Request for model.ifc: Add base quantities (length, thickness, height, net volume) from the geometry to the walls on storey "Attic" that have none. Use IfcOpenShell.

First a look at what the model holds.

```python
import ifcopenshell
import ifcopenshell.util.element
import ifcopenshell.util.unit

model = ifcopenshell.open("model.ifc")
print(model.schema)
for unit_type in ("LENGTHUNIT", "AREAUNIT", "VOLUMEUNIT"):
    print(unit_type, ifcopenshell.util.unit.calculate_unit_scale(model, unit_type))
storey = next(s for s in model.by_type("IfcBuildingStorey") if s.Name == "Attic")
walls = [e for e in ifcopenshell.util.element.get_decomposition(storey) if e.is_a("IfcWall")]
for e in sorted(walls, key=lambda e: e.id()):
    print(e.id(), e.is_a(), e.Name, list(ifcopenshell.util.element.get_psets(e, qtos_only=True)), sep=" | ")
```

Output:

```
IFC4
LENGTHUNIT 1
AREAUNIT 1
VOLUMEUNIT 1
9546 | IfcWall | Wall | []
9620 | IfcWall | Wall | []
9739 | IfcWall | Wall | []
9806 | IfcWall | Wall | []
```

```python
import ifcopenshell
import ifcopenshell.api.pset
import ifcopenshell.geom
import ifcopenshell.util.element
import ifcopenshell.util.shape
import ifcopenshell.util.unit

model = ifcopenshell.open("model.ifc")
unit_scale = ifcopenshell.util.unit.calculate_unit_scale(model)
volume_scale = ifcopenshell.util.unit.calculate_unit_scale(model, "VOLUMEUNIT")
settings = ifcopenshell.geom.settings()

storey = next(s for s in model.by_type("IfcBuildingStorey") if s.Name == "Attic")
walls = [e for e in ifcopenshell.util.element.get_decomposition(storey) if e.is_a("IfcWall")]

for e in sorted(walls, key=lambda e: e.id()):
    if ifcopenshell.util.element.get_psets(e, qtos_only=True, should_inherit=False):
        continue
    # Geometry comes back in metres, in the element's own axes.
    shape = ifcopenshell.geom.create_shape(settings, e)
    values = {
        "Length": ifcopenshell.util.shape.get_x(shape.geometry) / unit_scale,
        "Width": ifcopenshell.util.shape.get_y(shape.geometry) / unit_scale,
        "Height": ifcopenshell.util.shape.get_z(shape.geometry) / unit_scale,
        "NetVolume": ifcopenshell.util.shape.get_volume(shape.geometry) / volume_scale,
    }
    qto = ifcopenshell.api.pset.add_qto(model, product=e, name="Qto_WallBaseQuantities")
    ifcopenshell.api.pset.edit_qto(model, qto=qto, properties=values)
    print(e.id(), {k: round(v, 3) for k, v in values.items()})

model.write("model_edited.ifc")
```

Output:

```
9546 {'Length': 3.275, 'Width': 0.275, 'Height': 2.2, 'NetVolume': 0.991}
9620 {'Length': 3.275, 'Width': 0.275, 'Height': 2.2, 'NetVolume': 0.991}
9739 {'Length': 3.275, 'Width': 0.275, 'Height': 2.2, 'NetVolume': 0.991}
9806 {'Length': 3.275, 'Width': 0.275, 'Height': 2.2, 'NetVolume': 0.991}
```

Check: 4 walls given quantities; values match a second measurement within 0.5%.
